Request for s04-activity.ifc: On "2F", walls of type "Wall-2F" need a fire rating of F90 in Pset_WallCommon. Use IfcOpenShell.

First a look at what the model holds.

```python
import ifcopenshell
import ifcopenshell.util.element

model = ifcopenshell.open("s04-activity.ifc")
print(model.schema)
storey = next(s for s in model.by_type("IfcBuildingStorey") if s.Name == "2F")
walls = [e for e in ifcopenshell.util.element.get_decomposition(storey) if e.is_a("IfcWall")]
seen = {}
for e in walls:
    element_type = ifcopenshell.util.element.get_type(e)
    key = (element_type.Name if element_type != e and element_type else None, ifcopenshell.util.element.get_pset(e, "Pset_WallCommon", "FireRating"))
    seen[key] = seen.get(key, 0) + 1
for (name, value), count in sorted(seen.items(), key=str):
    print(count, "x", name, "|", value)
```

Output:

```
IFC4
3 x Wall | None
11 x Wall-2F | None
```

```python
import ifcopenshell
import ifcopenshell.api.pset
import ifcopenshell.util.element

model = ifcopenshell.open("s04-activity.ifc")

storey = next(s for s in model.by_type("IfcBuildingStorey") if s.Name == "2F")
walls = [e for e in ifcopenshell.util.element.get_decomposition(storey) if e.is_a("IfcWall")]

count = 0
for e in walls:
    element_type = ifcopenshell.util.element.get_type(e)
    if element_type in (None, e) or element_type.Name != "Wall-2F":
        continue
    # add_pset returns the element's existing set when there is one.
    pset = ifcopenshell.api.pset.add_pset(model, product=e, name="Pset_WallCommon")
    ifcopenshell.api.pset.edit_pset(model, pset=pset, properties={"FireRating": "F90"})
    count += 1

print(count, "walls updated")

model.write("s04-activity_edited.ifc")
```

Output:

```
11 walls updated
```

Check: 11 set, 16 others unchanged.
